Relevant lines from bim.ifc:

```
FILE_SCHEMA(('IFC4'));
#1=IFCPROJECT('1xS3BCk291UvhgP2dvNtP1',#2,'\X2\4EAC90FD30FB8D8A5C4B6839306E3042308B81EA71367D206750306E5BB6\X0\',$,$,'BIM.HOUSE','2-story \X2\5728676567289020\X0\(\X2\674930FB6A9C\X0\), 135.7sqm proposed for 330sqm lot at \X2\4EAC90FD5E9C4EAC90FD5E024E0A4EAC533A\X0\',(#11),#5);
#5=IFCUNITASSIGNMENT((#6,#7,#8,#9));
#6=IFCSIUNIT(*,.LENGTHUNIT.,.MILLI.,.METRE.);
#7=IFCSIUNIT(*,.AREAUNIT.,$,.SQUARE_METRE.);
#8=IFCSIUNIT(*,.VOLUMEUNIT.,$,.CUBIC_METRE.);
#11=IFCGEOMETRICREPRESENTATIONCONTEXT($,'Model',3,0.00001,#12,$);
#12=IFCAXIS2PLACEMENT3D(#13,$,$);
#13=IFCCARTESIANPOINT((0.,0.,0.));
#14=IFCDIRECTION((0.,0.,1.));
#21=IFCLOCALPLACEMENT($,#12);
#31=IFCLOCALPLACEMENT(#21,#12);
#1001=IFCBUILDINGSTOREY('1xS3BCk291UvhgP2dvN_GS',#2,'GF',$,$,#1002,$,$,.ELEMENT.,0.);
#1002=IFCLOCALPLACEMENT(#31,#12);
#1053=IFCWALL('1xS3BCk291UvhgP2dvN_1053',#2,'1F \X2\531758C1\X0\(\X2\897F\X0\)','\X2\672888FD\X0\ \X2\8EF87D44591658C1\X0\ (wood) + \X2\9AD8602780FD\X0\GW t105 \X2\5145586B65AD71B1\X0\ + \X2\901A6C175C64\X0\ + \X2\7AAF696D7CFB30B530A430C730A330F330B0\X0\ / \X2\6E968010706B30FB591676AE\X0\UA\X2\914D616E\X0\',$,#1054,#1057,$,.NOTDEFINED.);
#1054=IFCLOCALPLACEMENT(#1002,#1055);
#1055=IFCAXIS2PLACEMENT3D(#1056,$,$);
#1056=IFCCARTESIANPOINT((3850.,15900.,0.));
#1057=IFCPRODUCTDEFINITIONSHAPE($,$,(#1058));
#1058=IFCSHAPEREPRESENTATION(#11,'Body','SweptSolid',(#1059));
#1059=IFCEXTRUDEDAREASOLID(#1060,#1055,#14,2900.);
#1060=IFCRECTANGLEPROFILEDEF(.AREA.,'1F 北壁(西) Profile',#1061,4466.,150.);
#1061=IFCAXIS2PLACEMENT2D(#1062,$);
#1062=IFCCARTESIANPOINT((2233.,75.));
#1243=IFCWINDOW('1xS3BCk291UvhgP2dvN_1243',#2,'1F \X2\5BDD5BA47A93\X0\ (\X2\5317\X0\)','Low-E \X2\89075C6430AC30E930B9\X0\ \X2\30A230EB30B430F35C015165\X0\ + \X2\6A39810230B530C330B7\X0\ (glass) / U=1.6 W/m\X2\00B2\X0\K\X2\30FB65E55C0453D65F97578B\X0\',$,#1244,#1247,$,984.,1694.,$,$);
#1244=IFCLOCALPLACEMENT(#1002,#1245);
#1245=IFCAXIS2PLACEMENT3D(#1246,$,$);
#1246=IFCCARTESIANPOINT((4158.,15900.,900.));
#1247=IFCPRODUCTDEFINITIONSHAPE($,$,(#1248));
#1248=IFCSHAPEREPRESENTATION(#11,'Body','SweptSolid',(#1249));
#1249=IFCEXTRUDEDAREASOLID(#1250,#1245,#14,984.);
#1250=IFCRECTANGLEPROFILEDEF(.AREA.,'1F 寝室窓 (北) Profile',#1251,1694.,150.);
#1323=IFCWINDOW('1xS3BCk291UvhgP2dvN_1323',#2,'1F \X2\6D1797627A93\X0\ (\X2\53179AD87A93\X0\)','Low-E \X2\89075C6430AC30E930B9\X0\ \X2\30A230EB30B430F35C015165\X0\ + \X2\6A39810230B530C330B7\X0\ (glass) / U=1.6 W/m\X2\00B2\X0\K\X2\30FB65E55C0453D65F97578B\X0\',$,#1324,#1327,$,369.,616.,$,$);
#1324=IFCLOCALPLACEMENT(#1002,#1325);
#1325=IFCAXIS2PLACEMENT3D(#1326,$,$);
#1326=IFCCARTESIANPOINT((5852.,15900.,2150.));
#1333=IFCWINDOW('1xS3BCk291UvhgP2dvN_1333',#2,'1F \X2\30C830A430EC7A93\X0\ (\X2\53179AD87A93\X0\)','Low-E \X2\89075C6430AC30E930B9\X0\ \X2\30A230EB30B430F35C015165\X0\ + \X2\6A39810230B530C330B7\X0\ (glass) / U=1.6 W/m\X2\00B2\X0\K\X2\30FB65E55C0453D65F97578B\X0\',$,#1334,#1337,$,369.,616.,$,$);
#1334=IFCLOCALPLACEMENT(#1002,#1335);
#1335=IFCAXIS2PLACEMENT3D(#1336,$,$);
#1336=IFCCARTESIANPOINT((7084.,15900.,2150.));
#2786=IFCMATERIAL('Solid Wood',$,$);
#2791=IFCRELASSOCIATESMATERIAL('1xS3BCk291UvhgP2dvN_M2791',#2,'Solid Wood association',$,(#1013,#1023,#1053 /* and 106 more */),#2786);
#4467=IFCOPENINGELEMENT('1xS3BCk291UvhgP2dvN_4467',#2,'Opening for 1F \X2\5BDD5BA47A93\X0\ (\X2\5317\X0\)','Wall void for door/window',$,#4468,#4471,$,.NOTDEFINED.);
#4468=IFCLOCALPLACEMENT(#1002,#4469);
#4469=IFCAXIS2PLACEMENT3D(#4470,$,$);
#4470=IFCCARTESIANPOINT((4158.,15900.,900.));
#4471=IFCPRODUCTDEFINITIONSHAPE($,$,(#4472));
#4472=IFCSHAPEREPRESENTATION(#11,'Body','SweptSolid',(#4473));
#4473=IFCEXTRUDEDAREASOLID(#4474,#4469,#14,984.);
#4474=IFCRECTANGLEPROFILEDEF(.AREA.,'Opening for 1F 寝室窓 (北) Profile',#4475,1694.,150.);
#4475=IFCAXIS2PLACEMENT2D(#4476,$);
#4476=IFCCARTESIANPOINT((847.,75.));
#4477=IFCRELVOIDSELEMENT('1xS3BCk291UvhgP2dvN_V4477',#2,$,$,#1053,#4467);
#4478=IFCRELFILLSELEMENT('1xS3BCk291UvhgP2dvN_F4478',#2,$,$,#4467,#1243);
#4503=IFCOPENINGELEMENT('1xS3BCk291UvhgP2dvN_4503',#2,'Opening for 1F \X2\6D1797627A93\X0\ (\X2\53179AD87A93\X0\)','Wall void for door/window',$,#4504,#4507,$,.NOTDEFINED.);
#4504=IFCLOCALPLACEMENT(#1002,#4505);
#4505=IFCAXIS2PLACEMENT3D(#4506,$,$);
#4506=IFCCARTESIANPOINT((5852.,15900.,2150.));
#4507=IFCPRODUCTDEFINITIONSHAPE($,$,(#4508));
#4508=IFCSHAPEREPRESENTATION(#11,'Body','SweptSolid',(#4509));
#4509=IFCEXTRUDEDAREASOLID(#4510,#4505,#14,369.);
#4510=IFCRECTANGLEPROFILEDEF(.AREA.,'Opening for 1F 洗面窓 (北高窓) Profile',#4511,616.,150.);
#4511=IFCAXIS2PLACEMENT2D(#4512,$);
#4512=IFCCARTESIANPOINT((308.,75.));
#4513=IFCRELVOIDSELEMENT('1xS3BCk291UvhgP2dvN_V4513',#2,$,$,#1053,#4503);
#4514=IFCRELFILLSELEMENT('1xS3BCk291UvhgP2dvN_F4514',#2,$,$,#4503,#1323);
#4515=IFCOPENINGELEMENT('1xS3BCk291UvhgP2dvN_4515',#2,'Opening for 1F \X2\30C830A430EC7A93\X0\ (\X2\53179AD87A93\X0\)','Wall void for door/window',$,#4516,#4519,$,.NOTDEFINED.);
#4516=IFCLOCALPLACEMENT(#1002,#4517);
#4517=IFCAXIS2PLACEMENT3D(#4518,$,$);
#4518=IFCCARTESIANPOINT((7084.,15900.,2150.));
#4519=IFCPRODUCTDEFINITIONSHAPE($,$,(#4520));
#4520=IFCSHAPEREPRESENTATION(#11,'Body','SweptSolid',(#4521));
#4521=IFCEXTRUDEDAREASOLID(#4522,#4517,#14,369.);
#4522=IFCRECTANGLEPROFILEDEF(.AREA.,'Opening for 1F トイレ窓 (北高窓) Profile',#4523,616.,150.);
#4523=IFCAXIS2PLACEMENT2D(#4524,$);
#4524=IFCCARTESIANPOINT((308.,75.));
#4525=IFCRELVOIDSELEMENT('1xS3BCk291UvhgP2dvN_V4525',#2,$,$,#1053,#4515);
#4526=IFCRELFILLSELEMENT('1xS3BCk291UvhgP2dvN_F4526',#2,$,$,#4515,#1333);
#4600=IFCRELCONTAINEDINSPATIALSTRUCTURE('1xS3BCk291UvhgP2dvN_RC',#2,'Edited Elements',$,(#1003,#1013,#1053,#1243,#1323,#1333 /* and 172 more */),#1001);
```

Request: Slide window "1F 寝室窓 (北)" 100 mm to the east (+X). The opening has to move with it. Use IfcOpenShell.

```python
import ifcopenshell
import ifcopenshell.api.geometry
import ifcopenshell.util.placement

model = ifcopenshell.open("bim.ifc")

window = model.by_guid("1xS3BCk291UvhgP2dvN_1243")
opening = window.FillsVoids[0].RelatingOpeningElement
wall = opening.VoidsElements[0].RelatingBuildingElement

wall_matrix = ifcopenshell.util.placement.get_local_placement(wall.ObjectPlacement)
shift = wall_matrix[:3, 0] * 100.0
before = ifcopenshell.util.placement.get_local_placement(window.ObjectPlacement)[:3, 3].copy()

# The window is not placed relative to its opening, so move both.
for product in (opening, window):
    matrix = ifcopenshell.util.placement.get_local_placement(product.ObjectPlacement)
    matrix[:3, 3] += shift
    ifcopenshell.api.geometry.edit_object_placement(model, product=product, matrix=matrix, is_si=False)

after = ifcopenshell.util.placement.get_local_placement(window.ObjectPlacement)[:3, 3]
print("window moved by", (after - before).round(3) + 0.0)

model.write("bim-out.ifc")
```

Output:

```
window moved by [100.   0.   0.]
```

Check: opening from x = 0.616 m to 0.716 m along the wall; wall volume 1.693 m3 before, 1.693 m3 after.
